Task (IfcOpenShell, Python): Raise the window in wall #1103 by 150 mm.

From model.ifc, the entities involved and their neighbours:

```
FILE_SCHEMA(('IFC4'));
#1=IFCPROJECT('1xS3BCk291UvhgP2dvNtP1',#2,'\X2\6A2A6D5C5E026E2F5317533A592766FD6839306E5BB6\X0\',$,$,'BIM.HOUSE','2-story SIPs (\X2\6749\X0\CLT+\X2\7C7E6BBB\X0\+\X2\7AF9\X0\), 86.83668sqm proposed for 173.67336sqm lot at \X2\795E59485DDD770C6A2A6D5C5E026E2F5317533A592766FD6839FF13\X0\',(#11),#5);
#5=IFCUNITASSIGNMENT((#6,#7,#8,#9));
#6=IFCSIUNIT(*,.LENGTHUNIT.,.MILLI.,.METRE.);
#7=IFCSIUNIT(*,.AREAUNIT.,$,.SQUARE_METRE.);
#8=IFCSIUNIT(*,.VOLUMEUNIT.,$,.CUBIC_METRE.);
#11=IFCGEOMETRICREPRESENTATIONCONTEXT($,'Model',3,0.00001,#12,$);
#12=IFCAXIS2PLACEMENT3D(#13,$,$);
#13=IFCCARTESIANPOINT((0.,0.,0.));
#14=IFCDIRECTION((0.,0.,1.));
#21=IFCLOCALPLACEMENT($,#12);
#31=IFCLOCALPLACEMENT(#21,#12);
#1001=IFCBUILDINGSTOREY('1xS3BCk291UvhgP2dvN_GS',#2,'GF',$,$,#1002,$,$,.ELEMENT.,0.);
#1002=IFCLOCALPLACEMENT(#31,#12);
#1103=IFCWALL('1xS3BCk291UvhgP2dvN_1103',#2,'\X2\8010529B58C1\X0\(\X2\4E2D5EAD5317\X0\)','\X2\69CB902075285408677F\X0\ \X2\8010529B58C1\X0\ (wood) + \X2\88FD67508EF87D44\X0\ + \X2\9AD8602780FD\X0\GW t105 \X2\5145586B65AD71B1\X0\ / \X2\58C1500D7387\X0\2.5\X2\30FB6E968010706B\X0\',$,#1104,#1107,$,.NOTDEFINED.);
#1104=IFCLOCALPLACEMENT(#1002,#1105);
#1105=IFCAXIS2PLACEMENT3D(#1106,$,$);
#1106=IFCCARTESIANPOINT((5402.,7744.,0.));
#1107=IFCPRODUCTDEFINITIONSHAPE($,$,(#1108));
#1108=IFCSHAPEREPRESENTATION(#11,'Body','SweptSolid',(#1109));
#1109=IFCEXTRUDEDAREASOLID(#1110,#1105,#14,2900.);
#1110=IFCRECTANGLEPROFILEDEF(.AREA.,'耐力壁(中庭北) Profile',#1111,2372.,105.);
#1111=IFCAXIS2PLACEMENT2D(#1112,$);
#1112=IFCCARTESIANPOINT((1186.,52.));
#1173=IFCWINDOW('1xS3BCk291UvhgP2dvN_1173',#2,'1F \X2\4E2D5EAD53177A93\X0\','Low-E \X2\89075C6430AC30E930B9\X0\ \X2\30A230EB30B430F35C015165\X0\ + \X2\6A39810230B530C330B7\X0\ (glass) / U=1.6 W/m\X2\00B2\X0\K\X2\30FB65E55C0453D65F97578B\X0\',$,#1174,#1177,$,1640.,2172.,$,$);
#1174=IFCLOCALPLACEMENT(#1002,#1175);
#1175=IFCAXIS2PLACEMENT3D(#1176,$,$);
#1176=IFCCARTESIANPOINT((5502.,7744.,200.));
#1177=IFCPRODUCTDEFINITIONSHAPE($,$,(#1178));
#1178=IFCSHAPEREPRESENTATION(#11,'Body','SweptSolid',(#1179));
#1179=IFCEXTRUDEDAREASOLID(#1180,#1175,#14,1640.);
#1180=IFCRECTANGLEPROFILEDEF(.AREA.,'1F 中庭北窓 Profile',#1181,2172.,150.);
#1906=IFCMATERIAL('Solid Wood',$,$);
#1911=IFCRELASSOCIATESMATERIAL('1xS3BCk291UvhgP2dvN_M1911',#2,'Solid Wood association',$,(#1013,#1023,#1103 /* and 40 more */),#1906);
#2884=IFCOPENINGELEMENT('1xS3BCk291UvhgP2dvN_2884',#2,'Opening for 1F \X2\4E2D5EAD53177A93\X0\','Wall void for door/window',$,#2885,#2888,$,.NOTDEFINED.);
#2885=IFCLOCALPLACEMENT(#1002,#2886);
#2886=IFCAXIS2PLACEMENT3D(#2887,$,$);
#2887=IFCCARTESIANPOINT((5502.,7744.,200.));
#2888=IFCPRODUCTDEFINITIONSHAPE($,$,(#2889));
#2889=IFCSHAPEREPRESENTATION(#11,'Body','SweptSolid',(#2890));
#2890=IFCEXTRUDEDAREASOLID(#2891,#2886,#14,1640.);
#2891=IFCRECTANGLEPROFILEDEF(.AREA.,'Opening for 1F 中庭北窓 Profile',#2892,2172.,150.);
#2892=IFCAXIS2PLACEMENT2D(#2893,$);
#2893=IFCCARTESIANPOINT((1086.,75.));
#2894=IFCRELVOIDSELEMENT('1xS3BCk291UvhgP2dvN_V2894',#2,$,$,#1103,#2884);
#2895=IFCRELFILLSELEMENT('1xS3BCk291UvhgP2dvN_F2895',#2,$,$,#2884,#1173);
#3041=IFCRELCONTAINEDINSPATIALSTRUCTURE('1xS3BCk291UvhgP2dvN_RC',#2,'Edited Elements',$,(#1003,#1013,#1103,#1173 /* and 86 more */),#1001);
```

```python
import numpy as np
import ifcopenshell
import ifcopenshell.api.geometry
import ifcopenshell.util.placement
import ifcopenshell.util.unit

model = ifcopenshell.open("model.ifc")
unit_scale = ifcopenshell.util.unit.calculate_unit_scale(model)

window = model.by_guid("1xS3BCk291UvhgP2dvN_1173")
opening = window.FillsVoids[0].RelatingOpeningElement
dz = 150.0

shift = np.array([0.0, 0.0, dz])
# The window is not placed relative to its opening, so move both.
for product in (opening, window):
    matrix = ifcopenshell.util.placement.get_local_placement(product.ObjectPlacement)
    matrix[:3, 3] += shift
    ifcopenshell.api.geometry.edit_object_placement(model, product=product, matrix=matrix, is_si=False)

print(f"moved by {dz * unit_scale:+.3f} m")

model.write("model_edited.ifc")
```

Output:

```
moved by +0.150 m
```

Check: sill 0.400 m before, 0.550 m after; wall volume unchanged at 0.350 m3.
